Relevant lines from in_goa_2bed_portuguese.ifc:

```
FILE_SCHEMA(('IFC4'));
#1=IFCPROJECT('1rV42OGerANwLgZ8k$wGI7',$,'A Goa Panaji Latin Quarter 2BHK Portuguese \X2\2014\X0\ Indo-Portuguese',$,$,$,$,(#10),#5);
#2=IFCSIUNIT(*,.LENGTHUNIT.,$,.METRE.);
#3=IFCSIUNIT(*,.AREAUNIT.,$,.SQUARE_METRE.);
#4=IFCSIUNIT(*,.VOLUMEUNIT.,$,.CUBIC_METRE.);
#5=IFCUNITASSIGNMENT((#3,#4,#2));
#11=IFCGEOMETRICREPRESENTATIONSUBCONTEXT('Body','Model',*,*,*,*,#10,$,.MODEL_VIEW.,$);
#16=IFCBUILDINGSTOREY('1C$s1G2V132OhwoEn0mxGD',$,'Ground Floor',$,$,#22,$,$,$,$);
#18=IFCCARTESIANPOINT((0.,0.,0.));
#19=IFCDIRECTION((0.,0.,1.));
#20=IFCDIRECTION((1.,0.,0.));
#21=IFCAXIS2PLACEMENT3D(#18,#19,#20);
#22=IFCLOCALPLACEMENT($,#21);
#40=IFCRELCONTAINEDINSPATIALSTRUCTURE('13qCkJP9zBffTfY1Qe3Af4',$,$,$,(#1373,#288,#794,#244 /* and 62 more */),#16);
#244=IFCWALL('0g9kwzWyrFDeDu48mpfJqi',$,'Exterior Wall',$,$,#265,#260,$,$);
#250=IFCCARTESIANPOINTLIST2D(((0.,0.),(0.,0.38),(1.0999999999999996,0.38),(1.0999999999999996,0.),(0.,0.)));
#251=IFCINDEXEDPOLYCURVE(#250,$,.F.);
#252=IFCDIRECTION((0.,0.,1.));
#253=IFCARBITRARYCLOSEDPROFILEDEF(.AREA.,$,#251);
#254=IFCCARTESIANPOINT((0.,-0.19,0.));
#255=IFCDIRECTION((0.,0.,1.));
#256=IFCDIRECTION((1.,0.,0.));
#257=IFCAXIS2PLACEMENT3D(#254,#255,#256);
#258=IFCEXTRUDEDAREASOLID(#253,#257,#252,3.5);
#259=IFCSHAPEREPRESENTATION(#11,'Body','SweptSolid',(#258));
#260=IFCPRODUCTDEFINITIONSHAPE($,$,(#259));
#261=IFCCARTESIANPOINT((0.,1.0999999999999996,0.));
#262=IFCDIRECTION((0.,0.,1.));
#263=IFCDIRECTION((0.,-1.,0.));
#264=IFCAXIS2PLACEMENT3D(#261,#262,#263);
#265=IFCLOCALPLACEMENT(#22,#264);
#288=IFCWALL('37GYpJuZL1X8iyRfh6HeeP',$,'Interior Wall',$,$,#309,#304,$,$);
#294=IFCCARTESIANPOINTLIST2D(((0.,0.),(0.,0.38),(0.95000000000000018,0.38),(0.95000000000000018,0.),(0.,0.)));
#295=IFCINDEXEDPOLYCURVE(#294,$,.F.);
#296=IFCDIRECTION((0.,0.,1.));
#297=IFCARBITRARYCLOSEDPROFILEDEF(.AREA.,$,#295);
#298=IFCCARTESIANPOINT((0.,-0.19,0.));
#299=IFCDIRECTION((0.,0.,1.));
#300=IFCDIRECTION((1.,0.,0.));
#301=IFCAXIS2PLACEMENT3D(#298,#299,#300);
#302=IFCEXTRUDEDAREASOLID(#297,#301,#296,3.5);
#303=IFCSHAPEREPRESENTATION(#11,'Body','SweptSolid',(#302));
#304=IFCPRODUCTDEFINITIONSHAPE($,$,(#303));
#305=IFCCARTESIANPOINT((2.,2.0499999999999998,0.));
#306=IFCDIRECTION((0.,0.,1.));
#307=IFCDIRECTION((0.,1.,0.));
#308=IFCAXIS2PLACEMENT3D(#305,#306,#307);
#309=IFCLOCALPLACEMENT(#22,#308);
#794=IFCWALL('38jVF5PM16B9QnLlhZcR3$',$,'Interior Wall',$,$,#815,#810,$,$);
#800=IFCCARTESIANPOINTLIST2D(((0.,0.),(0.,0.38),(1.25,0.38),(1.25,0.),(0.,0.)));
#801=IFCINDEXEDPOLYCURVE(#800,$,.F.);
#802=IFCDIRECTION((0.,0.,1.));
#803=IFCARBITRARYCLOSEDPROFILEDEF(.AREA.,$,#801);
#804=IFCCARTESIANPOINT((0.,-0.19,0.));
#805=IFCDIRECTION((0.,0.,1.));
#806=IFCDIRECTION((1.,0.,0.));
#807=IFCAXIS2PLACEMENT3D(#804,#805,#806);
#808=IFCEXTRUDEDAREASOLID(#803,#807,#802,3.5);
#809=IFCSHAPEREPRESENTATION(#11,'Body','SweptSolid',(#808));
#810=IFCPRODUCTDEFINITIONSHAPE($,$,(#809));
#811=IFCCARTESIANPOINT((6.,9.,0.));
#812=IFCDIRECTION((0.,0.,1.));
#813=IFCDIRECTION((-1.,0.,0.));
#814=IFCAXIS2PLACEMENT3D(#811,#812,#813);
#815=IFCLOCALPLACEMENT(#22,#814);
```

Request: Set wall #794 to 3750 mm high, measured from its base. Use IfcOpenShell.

```python
import ifcopenshell
import ifcopenshell.geom
import ifcopenshell.util.representation
import ifcopenshell.util.shape

model = ifcopenshell.open("in_goa_2bed_portuguese.ifc")
settings = ifcopenshell.geom.settings()


def volume(element):
    """Net volume in cubic metres, openings subtracted."""
    shape = ifcopenshell.geom.create_shape(settings, element)
    return ifcopenshell.util.shape.get_volume(shape.geometry)


wall = model.by_guid("38jVF5PM16B9QnLlhZcR3$")
before = volume(wall)

body = ifcopenshell.util.representation.get_representation(wall, "Model", "Body")
solid = body.Items[0]
old_height = solid.Depth
solid.Depth = 3.75
after = volume(wall)

print(f"height {old_height:g} -> {solid.Depth:g}, volume {before:.3f} -> {after:.3f} m3")

model.write("in_goa_2bed_portuguese_rev.ifc")
```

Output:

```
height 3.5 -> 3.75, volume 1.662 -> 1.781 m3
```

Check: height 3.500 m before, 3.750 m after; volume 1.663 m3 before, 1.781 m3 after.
